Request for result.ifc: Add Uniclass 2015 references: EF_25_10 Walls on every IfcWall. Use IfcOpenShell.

First a look at what the model holds.

```python
import ifcopenshell

model = ifcopenshell.open("result.ifc")
print(model.schema)
print("classifications:", [c.Name for c in model.by_type("IfcClassification")])
for ifc_class in ("IfcDoor", "IfcRoof", "IfcStair", "IfcWall", "IfcWindow"):
    print(ifc_class, len(model.by_type(ifc_class)))
```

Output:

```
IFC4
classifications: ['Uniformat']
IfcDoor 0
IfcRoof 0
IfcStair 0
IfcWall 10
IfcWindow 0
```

```python
import ifcopenshell
import ifcopenshell.api.classification

model = ifcopenshell.open("result.ifc")

system = ifcopenshell.api.classification.add_classification(model, classification="Uniclass 2015")

codes = {
    "IfcWall": ("EF_25_10", "Walls"),
}
for ifc_class, (code, name) in codes.items():
    products = model.by_type(ifc_class)
    ifcopenshell.api.classification.add_reference(
        model, products=products, classification=system, identification=code, name=name
    )
    print(code, len(products))

model.write("result_rev.ifc")
```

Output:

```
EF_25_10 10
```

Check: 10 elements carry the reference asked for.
